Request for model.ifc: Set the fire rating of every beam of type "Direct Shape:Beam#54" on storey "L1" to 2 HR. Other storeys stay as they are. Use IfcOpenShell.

First a look at what the model holds.

```python
import ifcopenshell
import ifcopenshell.util.element

model = ifcopenshell.open("model.ifc")
print(model.schema)
storey = next(s for s in model.by_type("IfcBuildingStorey") if s.Name == "L1")
beams = [e for e in ifcopenshell.util.element.get_decomposition(storey) if e.is_a("IfcBeam")]
seen = {}
for e in beams:
    element_type = ifcopenshell.util.element.get_type(e)
    key = (element_type.Name if element_type != e and element_type else None, ifcopenshell.util.element.get_pset(e, "Pset_BeamCommon", "FireRating"))
    seen[key] = seen.get(key, 0) + 1
for (name, value), count in sorted(seen.items(), key=str):
    print(count, "x", name, "|", value)
```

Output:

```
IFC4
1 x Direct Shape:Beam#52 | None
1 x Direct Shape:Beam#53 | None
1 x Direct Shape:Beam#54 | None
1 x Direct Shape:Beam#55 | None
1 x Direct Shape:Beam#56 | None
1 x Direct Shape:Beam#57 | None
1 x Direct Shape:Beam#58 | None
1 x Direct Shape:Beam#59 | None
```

```python
import ifcopenshell
import ifcopenshell.api.pset
import ifcopenshell.util.element

model = ifcopenshell.open("model.ifc")

storey = next(s for s in model.by_type("IfcBuildingStorey") if s.Name == "L1")
beams = [e for e in ifcopenshell.util.element.get_decomposition(storey) if e.is_a("IfcBeam")]

count = 0
for e in beams:
    element_type = ifcopenshell.util.element.get_type(e)
    if element_type in (None, e) or element_type.Name != "Direct Shape:Beam#54":
        continue
    # add_pset returns the element's existing set when there is one.
    pset = ifcopenshell.api.pset.add_pset(model, product=e, name="Pset_BeamCommon")
    ifcopenshell.api.pset.edit_pset(model, pset=pset, properties={"FireRating": "2 HR"})
    count += 1

print(count, "beams updated")

model.write("model_v2.ifc")
```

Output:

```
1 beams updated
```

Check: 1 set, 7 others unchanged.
